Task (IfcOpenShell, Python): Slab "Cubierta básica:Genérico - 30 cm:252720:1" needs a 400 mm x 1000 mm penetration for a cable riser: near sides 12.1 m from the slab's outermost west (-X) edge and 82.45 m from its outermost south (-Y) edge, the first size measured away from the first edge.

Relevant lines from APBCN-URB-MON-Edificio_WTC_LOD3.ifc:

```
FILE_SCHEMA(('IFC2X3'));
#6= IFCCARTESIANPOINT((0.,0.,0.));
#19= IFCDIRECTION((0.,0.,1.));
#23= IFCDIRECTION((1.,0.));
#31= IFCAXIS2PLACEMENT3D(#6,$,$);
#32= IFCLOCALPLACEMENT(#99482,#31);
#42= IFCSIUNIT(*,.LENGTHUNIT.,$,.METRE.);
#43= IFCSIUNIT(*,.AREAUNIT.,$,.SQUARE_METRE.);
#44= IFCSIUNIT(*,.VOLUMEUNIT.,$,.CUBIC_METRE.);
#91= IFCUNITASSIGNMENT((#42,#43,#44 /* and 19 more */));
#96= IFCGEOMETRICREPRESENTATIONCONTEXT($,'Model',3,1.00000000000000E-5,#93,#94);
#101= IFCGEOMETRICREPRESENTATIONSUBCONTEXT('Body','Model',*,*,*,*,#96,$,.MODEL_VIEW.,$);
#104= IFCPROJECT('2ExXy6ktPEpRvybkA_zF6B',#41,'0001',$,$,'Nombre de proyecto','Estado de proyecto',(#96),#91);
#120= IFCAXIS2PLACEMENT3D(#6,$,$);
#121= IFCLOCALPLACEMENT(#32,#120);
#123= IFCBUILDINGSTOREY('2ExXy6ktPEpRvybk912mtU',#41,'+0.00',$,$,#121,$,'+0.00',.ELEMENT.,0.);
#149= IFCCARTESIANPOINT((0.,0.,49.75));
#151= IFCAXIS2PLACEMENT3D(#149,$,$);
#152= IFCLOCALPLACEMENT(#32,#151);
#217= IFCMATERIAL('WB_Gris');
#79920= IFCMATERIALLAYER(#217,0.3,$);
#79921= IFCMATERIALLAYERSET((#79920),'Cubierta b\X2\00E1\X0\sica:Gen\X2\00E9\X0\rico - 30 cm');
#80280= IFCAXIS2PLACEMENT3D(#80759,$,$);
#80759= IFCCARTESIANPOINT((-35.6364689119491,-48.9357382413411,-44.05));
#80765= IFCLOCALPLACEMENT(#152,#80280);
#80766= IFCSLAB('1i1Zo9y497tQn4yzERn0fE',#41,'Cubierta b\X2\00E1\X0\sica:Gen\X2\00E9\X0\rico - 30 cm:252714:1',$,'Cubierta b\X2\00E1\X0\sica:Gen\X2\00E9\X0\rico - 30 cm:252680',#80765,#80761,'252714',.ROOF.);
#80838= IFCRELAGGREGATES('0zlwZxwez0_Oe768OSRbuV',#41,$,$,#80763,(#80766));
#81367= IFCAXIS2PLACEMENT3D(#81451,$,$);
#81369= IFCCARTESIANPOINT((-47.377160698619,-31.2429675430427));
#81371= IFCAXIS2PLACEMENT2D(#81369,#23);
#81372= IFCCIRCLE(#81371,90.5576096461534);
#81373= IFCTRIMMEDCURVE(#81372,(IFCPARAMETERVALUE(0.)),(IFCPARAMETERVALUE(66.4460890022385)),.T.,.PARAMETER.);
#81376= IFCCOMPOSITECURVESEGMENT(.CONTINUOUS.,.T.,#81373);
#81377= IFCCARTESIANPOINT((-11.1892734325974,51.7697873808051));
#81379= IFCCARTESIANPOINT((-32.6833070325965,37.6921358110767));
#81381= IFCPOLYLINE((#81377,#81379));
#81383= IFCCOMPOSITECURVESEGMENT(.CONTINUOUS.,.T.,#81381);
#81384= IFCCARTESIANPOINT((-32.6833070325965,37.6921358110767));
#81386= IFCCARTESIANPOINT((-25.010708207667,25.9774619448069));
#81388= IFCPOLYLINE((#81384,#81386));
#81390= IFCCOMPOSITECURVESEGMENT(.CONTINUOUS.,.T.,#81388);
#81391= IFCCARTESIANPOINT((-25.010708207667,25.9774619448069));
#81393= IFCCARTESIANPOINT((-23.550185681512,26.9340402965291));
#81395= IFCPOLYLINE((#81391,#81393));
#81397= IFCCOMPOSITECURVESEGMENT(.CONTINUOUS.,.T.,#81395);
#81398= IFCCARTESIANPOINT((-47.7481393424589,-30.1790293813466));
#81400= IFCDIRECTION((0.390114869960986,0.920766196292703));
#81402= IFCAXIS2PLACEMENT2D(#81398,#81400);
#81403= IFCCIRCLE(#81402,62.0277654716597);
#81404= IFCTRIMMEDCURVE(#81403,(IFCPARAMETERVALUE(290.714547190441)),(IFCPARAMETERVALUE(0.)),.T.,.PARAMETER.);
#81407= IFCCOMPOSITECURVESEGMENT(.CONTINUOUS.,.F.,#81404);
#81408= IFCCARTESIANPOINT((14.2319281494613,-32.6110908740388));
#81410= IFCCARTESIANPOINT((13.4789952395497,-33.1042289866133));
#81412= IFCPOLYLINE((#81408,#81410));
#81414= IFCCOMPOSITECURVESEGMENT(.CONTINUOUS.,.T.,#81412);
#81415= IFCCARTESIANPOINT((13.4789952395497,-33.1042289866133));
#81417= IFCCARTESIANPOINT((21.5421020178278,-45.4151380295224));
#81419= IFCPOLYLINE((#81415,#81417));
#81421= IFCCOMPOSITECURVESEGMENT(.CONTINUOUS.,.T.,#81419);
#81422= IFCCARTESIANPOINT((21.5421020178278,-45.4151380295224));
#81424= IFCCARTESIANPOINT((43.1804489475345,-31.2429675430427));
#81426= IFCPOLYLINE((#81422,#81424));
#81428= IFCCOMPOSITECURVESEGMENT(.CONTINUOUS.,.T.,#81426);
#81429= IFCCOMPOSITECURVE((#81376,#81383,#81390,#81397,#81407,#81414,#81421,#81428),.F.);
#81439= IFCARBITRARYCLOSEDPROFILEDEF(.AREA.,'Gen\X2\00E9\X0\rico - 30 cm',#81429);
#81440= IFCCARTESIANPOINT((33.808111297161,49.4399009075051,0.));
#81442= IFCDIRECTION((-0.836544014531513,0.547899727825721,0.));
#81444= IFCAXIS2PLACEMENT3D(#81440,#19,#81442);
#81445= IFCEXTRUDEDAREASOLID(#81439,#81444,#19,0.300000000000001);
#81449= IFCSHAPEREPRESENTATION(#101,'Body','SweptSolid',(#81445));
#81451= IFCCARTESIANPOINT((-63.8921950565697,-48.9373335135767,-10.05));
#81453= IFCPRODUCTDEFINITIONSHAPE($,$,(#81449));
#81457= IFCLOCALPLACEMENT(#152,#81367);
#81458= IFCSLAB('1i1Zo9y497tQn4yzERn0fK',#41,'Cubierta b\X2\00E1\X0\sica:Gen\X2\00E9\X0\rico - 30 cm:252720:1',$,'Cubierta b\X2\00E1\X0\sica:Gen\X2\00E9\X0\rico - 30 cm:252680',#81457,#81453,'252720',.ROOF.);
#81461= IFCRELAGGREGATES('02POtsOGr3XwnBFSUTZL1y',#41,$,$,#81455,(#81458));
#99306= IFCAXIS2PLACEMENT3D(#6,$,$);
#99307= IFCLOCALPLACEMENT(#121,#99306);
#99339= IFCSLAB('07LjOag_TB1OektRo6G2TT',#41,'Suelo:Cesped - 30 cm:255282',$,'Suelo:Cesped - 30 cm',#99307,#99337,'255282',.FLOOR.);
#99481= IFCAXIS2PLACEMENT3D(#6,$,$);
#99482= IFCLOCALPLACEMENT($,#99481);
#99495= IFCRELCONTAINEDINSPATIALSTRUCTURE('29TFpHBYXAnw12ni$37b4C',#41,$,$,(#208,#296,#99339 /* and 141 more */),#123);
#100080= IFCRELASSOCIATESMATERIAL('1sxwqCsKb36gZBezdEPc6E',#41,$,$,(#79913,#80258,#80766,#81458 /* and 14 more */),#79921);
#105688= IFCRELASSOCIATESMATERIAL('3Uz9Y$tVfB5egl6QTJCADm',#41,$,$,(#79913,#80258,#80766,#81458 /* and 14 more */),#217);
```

```python
import numpy as np
import ifcopenshell
import ifcopenshell.api.feature
import ifcopenshell.api.geometry
import ifcopenshell.api.root
import ifcopenshell.geom
import ifcopenshell.util.placement
import ifcopenshell.util.representation
import ifcopenshell.util.shape
import ifcopenshell.util.unit

model = ifcopenshell.open("APBCN-URB-MON-Edificio_WTC_LOD3.ifc")
unit_scale = ifcopenshell.util.unit.calculate_unit_scale(model)
settings = ifcopenshell.geom.settings()


def volume(element):
    """Net volume in cubic metres, openings subtracted."""
    shape = ifcopenshell.geom.create_shape(settings, element)
    return ifcopenshell.util.shape.get_volume(shape.geometry)


slab = model.by_id(81458)
before = volume(slab)

# Extent in the slab's own axes, in metres. The edges named are its -X and -Y sides.
slab_shape = ifcopenshell.geom.create_shape(settings, slab)
vertices = ifcopenshell.util.shape.get_vertices(slab_shape.geometry)
x_min, y_min, bottom = vertices.min(axis=0)
top = vertices[:, 2].max()

opening = ifcopenshell.api.root.create_entity(model, ifc_class="IfcOpeningElement", name="Cable riser opening")
context = ifcopenshell.util.representation.get_context(model, "Model", "Body", "MODEL_VIEW")
width, depth = 0.4, 1
outline = [(0.0, 0.0), (width, 0.0), (width, depth), (0.0, depth), (0.0, 0.0)]
# Overshoot both faces by 50 mm so the cut is clean.
shape = ifcopenshell.api.geometry.add_slab_representation(
    model, context=context, depth=top - bottom + 0.1, polyline=outline
)
ifcopenshell.api.geometry.assign_representation(model, product=opening, representation=shape)

matrix = ifcopenshell.util.placement.get_local_placement(slab.ObjectPlacement)
matrix[:, 3] = matrix @ np.append(np.array([x_min + 12.1, y_min + 82.45, bottom - 0.05]) / unit_scale, 1.0)
ifcopenshell.api.geometry.edit_object_placement(model, product=opening, matrix=matrix, is_si=False)
ifcopenshell.api.feature.add_feature(model, feature=opening, element=slab)

after = volume(slab)

print(f"slab volume {before:.3f} -> {after:.3f} m3")

model.write("APBCN-URB-MON-Edificio_WTC_LOD3-out.ifc")
```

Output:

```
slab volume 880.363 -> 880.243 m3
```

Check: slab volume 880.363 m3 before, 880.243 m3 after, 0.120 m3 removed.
